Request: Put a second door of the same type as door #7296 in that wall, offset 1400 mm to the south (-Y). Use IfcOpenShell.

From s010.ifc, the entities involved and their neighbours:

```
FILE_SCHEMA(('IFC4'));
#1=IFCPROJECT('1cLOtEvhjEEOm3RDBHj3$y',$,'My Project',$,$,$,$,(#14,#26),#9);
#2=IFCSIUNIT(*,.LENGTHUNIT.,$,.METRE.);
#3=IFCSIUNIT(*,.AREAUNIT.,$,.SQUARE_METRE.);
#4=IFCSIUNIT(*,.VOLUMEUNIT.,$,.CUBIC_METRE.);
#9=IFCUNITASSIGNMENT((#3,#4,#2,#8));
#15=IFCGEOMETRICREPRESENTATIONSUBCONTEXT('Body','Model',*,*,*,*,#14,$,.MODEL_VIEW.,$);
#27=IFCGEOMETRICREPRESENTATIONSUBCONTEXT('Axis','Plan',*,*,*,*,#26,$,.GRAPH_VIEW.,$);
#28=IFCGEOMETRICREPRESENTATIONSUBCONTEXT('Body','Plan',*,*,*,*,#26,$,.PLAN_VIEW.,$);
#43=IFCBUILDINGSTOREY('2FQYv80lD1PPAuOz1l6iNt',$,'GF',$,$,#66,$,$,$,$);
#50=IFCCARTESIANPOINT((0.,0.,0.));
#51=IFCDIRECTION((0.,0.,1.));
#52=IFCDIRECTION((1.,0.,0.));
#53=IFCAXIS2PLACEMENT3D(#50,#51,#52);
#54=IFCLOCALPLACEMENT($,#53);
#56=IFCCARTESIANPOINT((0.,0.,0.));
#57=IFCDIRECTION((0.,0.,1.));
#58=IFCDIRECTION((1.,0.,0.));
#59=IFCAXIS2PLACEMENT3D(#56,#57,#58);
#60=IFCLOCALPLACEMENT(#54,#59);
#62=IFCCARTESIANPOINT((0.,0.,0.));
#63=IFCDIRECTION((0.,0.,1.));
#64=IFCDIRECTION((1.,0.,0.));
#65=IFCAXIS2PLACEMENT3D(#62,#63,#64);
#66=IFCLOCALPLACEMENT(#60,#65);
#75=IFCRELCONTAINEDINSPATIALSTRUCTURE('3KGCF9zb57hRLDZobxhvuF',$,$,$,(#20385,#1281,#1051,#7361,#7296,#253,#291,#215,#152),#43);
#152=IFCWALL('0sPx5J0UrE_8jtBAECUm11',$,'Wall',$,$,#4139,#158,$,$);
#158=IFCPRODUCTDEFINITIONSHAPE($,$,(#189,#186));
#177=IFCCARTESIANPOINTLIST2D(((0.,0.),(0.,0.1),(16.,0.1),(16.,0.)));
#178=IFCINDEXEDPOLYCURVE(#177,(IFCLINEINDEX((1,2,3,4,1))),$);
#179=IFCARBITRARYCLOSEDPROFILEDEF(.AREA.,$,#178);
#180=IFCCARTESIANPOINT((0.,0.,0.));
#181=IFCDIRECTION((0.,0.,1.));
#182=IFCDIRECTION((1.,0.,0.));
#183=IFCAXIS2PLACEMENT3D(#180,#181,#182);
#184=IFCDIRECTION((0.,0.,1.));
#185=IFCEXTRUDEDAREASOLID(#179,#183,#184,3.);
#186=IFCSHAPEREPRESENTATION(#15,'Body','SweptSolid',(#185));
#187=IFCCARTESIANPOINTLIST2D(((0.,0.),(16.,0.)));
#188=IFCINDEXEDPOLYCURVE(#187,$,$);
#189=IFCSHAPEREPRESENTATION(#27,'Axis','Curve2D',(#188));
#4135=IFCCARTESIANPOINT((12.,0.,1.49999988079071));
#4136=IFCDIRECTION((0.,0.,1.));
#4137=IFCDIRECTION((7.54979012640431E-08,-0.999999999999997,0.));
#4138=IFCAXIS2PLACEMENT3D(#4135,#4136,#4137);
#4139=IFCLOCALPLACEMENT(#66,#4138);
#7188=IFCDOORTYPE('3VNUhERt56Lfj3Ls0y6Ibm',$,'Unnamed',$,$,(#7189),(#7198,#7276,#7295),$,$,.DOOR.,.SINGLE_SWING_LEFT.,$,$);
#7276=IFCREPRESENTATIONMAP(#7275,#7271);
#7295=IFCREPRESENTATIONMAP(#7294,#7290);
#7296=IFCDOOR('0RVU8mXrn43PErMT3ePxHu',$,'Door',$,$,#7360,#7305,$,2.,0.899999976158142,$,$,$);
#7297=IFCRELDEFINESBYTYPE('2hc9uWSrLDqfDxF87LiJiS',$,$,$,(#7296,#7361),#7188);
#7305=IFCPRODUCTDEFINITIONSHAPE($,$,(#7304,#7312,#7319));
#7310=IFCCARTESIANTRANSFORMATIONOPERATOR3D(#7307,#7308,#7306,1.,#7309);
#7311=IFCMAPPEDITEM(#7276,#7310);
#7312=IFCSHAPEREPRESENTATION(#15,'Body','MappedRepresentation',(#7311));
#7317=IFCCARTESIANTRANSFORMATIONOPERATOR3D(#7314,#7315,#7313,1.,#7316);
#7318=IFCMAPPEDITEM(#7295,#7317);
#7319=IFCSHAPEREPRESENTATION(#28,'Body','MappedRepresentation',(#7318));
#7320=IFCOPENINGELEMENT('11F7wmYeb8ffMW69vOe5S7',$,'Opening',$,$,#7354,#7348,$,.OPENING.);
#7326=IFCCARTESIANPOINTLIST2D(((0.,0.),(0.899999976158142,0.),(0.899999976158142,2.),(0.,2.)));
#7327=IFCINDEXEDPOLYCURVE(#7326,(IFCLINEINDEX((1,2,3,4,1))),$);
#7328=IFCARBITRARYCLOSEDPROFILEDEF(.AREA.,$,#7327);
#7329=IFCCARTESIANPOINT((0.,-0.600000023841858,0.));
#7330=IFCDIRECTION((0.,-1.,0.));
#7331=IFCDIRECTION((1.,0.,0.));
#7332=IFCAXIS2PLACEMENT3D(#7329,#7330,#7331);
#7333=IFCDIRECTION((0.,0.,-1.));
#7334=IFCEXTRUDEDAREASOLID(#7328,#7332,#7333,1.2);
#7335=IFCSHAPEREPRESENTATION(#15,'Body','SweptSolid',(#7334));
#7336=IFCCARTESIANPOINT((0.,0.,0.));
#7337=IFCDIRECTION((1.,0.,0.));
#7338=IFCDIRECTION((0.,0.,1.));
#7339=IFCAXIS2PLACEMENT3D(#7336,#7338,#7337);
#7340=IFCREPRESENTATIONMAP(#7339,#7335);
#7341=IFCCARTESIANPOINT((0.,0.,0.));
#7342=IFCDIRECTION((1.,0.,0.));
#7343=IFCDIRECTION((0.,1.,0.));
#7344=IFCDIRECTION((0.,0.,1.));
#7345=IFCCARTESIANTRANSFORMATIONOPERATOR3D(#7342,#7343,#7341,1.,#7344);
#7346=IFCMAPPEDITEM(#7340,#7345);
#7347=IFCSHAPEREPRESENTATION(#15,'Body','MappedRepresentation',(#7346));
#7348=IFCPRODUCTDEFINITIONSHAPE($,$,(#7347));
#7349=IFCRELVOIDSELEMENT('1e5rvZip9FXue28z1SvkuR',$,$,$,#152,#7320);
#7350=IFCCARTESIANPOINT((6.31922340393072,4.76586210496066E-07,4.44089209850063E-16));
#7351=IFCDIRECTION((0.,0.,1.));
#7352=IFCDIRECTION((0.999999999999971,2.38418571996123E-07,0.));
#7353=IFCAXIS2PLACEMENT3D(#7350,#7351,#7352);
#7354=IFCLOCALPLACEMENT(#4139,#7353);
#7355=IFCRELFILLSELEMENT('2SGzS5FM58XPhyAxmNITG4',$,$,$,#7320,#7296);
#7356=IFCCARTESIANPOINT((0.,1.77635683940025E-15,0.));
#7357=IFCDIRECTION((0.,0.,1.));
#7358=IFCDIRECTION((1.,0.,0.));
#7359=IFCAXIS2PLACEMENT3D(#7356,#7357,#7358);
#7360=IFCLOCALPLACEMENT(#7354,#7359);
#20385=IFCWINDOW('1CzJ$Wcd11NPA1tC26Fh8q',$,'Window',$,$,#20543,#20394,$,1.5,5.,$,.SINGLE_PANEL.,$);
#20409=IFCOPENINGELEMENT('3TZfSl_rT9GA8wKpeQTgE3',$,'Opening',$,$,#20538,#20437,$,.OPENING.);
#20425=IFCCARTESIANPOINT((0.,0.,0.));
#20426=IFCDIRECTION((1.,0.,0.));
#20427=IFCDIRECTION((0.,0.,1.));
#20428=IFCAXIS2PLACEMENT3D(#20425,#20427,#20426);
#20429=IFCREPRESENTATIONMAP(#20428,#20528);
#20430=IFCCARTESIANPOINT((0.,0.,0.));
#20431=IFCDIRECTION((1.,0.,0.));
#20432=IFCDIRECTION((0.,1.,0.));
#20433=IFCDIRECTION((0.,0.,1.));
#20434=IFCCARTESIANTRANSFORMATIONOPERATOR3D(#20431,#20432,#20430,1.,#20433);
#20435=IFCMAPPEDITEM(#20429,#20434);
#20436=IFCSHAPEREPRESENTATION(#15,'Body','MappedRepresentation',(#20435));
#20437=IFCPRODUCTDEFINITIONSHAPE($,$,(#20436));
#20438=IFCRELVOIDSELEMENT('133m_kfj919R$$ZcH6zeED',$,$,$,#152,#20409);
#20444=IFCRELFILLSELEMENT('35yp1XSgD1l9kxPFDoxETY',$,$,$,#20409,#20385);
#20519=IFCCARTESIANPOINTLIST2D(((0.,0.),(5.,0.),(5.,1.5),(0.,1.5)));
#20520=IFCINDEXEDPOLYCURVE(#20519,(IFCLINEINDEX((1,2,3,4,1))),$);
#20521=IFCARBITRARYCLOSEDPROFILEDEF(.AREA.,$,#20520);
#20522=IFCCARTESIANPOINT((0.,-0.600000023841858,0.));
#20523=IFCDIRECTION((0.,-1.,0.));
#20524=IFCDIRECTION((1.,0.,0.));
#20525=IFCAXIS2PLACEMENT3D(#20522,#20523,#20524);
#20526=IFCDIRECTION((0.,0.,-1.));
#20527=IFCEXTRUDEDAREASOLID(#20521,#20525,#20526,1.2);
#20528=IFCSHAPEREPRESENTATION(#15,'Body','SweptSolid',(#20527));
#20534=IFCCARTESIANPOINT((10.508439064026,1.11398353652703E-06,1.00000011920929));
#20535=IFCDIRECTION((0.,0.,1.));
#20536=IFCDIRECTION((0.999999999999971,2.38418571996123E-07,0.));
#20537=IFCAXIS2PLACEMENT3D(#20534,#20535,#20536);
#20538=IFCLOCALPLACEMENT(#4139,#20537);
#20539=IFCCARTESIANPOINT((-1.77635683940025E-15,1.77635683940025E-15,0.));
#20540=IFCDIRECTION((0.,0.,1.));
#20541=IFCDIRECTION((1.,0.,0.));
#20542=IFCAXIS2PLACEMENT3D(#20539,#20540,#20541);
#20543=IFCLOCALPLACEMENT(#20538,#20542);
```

```python
import ifcopenshell
import ifcopenshell.api.feature
import ifcopenshell.api.geometry
import ifcopenshell.api.root
import ifcopenshell.geom
import ifcopenshell.util.element
import ifcopenshell.util.placement
import ifcopenshell.util.shape
import ifcopenshell.util.unit

model = ifcopenshell.open("s010.ifc")
unit_scale = ifcopenshell.util.unit.calculate_unit_scale(model)
settings = ifcopenshell.geom.settings()


def volume(element):
    """Net volume in cubic metres, openings subtracted."""
    shape = ifcopenshell.geom.create_shape(settings, element)
    return ifcopenshell.util.shape.get_volume(shape.geometry)


door = model.by_guid("0RVU8mXrn43PErMT3ePxHu")
opening = door.FillsVoids[0].RelatingOpeningElement
wall = opening.VoidsElements[0].RelatingBuildingElement
before = volume(wall)
shift = ifcopenshell.util.placement.get_local_placement(wall.ObjectPlacement)[:3, 0] * 1.4 / unit_scale

# copy_class copies the void relationship, type, container and properties, but no geometry.
new_opening = ifcopenshell.api.root.copy_class(model, product=opening)
new_opening.Representation = ifcopenshell.util.element.copy_deep(
    model, opening.Representation, exclude=["IfcGeometricRepresentationContext", "IfcRepresentationMap"]
)
new_door = ifcopenshell.api.root.copy_class(model, product=door)
new_door.Representation = ifcopenshell.util.element.copy_deep(
    model, door.Representation, exclude=["IfcGeometricRepresentationContext", "IfcRepresentationMap"]
)
ifcopenshell.api.feature.add_filling(model, opening=new_opening, element=new_door)

for old, new in ((opening, new_opening), (door, new_door)):
    matrix = ifcopenshell.util.placement.get_local_placement(old.ObjectPlacement)
    matrix[:3, 3] += shift
    ifcopenshell.api.geometry.edit_object_placement(model, product=new, matrix=matrix, is_si=False)

after = volume(wall)

print(f"wall volume {before:.3f} -> {after:.3f} m3")

model.write("s010_rev.ifc")
```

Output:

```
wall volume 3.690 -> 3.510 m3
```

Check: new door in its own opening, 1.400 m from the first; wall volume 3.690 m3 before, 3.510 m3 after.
